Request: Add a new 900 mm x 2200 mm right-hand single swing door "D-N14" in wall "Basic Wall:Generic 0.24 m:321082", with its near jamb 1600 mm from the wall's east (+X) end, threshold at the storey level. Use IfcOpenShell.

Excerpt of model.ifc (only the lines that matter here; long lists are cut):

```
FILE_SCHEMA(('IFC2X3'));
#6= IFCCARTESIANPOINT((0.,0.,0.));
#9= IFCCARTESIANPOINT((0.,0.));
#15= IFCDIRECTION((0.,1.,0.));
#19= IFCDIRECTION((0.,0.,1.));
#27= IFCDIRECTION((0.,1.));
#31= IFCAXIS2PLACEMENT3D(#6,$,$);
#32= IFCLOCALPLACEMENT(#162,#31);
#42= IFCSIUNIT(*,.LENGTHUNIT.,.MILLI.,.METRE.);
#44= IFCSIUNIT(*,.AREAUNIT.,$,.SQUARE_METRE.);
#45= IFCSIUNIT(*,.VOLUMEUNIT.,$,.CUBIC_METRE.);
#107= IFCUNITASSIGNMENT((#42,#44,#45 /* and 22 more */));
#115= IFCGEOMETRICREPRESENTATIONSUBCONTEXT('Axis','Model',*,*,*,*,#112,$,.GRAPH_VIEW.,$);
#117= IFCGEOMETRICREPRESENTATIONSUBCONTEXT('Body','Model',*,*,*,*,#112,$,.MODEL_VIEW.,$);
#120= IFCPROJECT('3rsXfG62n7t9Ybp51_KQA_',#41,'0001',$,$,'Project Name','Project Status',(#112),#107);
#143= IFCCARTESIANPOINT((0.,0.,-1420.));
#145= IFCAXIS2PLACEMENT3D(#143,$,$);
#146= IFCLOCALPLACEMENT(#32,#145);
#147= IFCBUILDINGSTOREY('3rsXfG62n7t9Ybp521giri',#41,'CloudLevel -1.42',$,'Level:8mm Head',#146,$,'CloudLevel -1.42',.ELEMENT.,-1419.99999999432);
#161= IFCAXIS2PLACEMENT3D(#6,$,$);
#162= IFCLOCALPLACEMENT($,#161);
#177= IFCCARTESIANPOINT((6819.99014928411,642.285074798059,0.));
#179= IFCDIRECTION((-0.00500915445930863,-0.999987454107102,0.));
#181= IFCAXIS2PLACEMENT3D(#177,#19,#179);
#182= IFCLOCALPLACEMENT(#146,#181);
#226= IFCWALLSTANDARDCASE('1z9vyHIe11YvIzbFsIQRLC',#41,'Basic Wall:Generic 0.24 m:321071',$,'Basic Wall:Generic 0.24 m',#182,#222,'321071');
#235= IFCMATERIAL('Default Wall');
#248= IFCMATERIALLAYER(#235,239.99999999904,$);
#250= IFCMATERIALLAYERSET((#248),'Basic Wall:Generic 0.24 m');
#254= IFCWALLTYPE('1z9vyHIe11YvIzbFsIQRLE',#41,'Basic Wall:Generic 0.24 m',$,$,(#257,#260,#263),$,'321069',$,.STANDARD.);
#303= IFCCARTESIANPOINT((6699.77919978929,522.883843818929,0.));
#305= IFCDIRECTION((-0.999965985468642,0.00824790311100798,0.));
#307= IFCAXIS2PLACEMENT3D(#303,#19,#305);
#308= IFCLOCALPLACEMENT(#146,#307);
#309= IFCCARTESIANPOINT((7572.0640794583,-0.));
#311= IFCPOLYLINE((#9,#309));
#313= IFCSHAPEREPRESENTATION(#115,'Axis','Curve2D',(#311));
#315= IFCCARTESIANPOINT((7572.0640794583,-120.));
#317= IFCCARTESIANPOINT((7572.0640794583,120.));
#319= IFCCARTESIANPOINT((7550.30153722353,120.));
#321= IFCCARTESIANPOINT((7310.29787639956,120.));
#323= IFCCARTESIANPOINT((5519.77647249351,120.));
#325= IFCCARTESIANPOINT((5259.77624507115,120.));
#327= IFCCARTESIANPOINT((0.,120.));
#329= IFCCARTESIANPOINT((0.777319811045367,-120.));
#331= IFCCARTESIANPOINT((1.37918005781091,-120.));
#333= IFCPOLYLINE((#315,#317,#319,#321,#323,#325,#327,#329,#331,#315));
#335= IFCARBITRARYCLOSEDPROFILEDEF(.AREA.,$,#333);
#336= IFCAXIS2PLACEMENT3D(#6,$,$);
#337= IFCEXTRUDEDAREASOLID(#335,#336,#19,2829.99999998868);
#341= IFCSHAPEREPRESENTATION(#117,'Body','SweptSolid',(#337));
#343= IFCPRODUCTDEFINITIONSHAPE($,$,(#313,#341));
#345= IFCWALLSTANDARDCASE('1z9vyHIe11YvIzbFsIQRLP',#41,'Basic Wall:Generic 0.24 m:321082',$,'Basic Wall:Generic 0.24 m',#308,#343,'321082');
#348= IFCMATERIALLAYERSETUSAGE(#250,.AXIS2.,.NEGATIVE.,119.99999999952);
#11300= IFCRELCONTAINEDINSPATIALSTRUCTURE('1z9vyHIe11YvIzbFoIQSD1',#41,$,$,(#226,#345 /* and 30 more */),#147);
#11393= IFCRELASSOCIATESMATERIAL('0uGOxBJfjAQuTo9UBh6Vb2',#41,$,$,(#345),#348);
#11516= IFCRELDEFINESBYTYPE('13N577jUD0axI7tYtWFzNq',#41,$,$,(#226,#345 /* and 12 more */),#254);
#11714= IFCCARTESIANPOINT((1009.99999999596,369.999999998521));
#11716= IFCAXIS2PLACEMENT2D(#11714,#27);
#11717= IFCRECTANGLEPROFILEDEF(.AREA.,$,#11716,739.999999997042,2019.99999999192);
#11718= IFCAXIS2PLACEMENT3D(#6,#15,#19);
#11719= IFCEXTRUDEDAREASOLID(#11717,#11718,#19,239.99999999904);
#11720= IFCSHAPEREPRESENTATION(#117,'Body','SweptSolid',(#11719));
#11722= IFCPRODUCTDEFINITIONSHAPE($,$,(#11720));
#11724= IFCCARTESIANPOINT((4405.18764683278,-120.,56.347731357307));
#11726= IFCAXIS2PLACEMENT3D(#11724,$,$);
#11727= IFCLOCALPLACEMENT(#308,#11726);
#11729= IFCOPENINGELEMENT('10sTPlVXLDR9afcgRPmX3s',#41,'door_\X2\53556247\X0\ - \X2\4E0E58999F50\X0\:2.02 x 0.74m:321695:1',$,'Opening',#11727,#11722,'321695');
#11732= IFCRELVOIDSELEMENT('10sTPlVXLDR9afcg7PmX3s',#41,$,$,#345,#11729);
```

```python
import numpy as np
import ifcopenshell
import ifcopenshell.api.feature
import ifcopenshell.api.geometry
import ifcopenshell.api.root
import ifcopenshell.api.spatial
import ifcopenshell.api.type
import ifcopenshell.geom
import ifcopenshell.util.element
import ifcopenshell.util.placement
import ifcopenshell.util.representation
import ifcopenshell.util.shape
import ifcopenshell.util.unit

model = ifcopenshell.open("model.ifc")
unit_scale = ifcopenshell.util.unit.calculate_unit_scale(model)
settings = ifcopenshell.geom.settings()


def volume(element):
    """Net volume in cubic metres, openings subtracted."""
    shape = ifcopenshell.geom.create_shape(settings, element)
    return ifcopenshell.util.shape.get_volume(shape.geometry)


wall = model.by_guid("1z9vyHIe11YvIzbFsIQRLP")
storey = ifcopenshell.util.element.get_container(wall, ifc_class="IfcBuildingStorey")
context = ifcopenshell.util.representation.get_context(model, "Model", "Body", "MODEL_VIEW")
before = volume(wall)

width, height, from_end, sill = 0.9, 2.2, 1.6, 0.0  # metres

# The wall runs along its own X axis, and the end named is its -X end.
wall_shape = ifcopenshell.geom.create_shape(settings, wall)
x, y, z = ifcopenshell.util.shape.get_vertices(wall_shape.geometry).T
start = x.min() + from_end
face, thickness = float(y.min()), float(y.max() - y.min())
wall_matrix = ifcopenshell.util.placement.get_local_placement(wall.ObjectPlacement)
level = ifcopenshell.util.placement.get_local_placement(storey.ObjectPlacement)[2, 3]


def in_wall(x, y):
    """Placement at x, y metres in the wall's axes, at sill height."""
    matrix = wall_matrix.copy()
    matrix[:, 3] = wall_matrix @ np.array([x / unit_scale, y / unit_scale, 0.0, 1.0])
    matrix[2, 3] = level + sill / unit_scale
    return matrix


# Opening: a box that overshoots both wall faces by 50 mm.
opening = ifcopenshell.api.root.create_entity(model, ifc_class="IfcOpeningElement")
box = ifcopenshell.api.geometry.add_wall_representation(
    model, context=context, length=width, height=height, thickness=thickness + 0.1
)
ifcopenshell.api.geometry.assign_representation(model, product=opening, representation=box)
ifcopenshell.api.geometry.edit_object_placement(model, product=opening, matrix=in_wall(start, face - 0.05), is_si=False)
ifcopenshell.api.feature.add_feature(model, feature=opening, element=wall)

door = ifcopenshell.api.root.create_entity(model, ifc_class="IfcDoor", name="D-N14")
door.OverallWidth, door.OverallHeight = width / unit_scale, height / unit_scale
body = ifcopenshell.api.geometry.add_door_representation(
    model,
    context=context,
    overall_width=door.OverallWidth,
    overall_height=door.OverallHeight,
    operation_type="SINGLE_SWING_RIGHT",
    lining_properties={"LiningDepth": thickness / unit_scale, "ThresholdDepth": thickness / unit_scale},
)
ifcopenshell.api.geometry.assign_representation(model, product=door, representation=body)
ifcopenshell.api.spatial.assign_container(model, products=[door], relating_structure=storey)
fills = ifcopenshell.api.feature.add_filling(model, opening=opening, element=door)
fills.OwnerHistory = door.OwnerHistory  # required in IFC2X3

# IFC2X3 keeps the operation on the door style.
style = ifcopenshell.api.root.create_entity(model, ifc_class="IfcDoorStyle", name="D-N14")
style.OperationType, style.ConstructionType = "SINGLE_SWING_RIGHT", "NOTDEFINED"
style.ParameterTakesPrecedence = style.Sizeable = False
ifcopenshell.api.type.assign_type(model, related_objects=[door], relating_type=style)

# The lining spans the wall, so the door starts at the wall face.
ifcopenshell.api.geometry.edit_object_placement(model, product=door, matrix=in_wall(start, face), is_si=False)

after = volume(wall)

print(f"wall volume {before:.3f} -> {after:.3f} m3")

model.write("model_v2.ifc")
```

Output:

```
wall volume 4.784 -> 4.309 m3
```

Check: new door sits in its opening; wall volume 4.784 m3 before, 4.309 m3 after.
